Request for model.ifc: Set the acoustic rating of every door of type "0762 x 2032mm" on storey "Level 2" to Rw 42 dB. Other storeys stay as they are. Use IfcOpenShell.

First a look at what the model holds.

```python
import ifcopenshell
import ifcopenshell.util.element

model = ifcopenshell.open("model.ifc")
print(model.schema)
storey = next(s for s in model.by_type("IfcBuildingStorey") if s.Name == "Level 2")
doors = [e for e in ifcopenshell.util.element.get_decomposition(storey) if e.is_a("IfcDoor")]
seen = {}
for e in doors:
    element_type = ifcopenshell.util.element.get_type(e)
    key = (element_type.Name if element_type != e and element_type else None, ifcopenshell.util.element.get_pset(e, "Pset_DoorCommon", "AcousticRating"))
    seen[key] = seen.get(key, 0) + 1
for (name, value), count in sorted(seen.items(), key=str):
    print(count, "x", name, "|", value)
```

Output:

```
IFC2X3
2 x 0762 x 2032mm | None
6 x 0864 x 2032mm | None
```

```python
import ifcopenshell
import ifcopenshell.api.pset
import ifcopenshell.util.element

model = ifcopenshell.open("model.ifc")

storey = next(s for s in model.by_type("IfcBuildingStorey") if s.Name == "Level 2")
doors = [e for e in ifcopenshell.util.element.get_decomposition(storey) if e.is_a("IfcDoor")]

count = 0
for e in doors:
    element_type = ifcopenshell.util.element.get_type(e)
    if element_type in (None, e) or element_type.Name != "0762 x 2032mm":
        continue
    # add_pset returns the element's existing set when there is one.
    pset = ifcopenshell.api.pset.add_pset(model, product=e, name="Pset_DoorCommon")
    ifcopenshell.api.pset.edit_pset(model, pset=pset, properties={"AcousticRating": "Rw 42 dB"})
    count += 1

print(count, "doors updated")

model.write("model-out.ifc")
```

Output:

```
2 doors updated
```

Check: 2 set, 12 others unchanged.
